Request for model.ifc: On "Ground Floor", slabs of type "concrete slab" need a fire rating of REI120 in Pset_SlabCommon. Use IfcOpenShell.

First a look at what the model holds.

```python
import ifcopenshell
import ifcopenshell.util.element

model = ifcopenshell.open("model.ifc")
print(model.schema)
storey = next(s for s in model.by_type("IfcBuildingStorey") if s.Name == "Ground Floor")
slabs = [e for e in ifcopenshell.util.element.get_decomposition(storey) if e.is_a("IfcSlab")]
seen = {}
for e in slabs:
    element_type = ifcopenshell.util.element.get_type(e)
    key = (element_type.Name if element_type != e and element_type else None, ifcopenshell.util.element.get_pset(e, "Pset_SlabCommon", "FireRating"))
    seen[key] = seen.get(key, 0) + 1
for (name, value), count in sorted(seen.items(), key=str):
    print(count, "x", name, "|", value)
```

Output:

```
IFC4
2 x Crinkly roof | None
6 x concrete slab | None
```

```python
import ifcopenshell
import ifcopenshell.api.pset
import ifcopenshell.util.element

model = ifcopenshell.open("model.ifc")

storey = next(s for s in model.by_type("IfcBuildingStorey") if s.Name == "Ground Floor")
slabs = [e for e in ifcopenshell.util.element.get_decomposition(storey) if e.is_a("IfcSlab")]

count = 0
for e in slabs:
    element_type = ifcopenshell.util.element.get_type(e)
    if element_type in (None, e) or element_type.Name != "concrete slab":
        continue
    # add_pset returns the element's existing set when there is one.
    pset = ifcopenshell.api.pset.add_pset(model, product=e, name="Pset_SlabCommon")
    ifcopenshell.api.pset.edit_pset(model, pset=pset, properties={"FireRating": "REI120"})
    count += 1

print(count, "slabs updated")

model.write("model_v2.ifc")
```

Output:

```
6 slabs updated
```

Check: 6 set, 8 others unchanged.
